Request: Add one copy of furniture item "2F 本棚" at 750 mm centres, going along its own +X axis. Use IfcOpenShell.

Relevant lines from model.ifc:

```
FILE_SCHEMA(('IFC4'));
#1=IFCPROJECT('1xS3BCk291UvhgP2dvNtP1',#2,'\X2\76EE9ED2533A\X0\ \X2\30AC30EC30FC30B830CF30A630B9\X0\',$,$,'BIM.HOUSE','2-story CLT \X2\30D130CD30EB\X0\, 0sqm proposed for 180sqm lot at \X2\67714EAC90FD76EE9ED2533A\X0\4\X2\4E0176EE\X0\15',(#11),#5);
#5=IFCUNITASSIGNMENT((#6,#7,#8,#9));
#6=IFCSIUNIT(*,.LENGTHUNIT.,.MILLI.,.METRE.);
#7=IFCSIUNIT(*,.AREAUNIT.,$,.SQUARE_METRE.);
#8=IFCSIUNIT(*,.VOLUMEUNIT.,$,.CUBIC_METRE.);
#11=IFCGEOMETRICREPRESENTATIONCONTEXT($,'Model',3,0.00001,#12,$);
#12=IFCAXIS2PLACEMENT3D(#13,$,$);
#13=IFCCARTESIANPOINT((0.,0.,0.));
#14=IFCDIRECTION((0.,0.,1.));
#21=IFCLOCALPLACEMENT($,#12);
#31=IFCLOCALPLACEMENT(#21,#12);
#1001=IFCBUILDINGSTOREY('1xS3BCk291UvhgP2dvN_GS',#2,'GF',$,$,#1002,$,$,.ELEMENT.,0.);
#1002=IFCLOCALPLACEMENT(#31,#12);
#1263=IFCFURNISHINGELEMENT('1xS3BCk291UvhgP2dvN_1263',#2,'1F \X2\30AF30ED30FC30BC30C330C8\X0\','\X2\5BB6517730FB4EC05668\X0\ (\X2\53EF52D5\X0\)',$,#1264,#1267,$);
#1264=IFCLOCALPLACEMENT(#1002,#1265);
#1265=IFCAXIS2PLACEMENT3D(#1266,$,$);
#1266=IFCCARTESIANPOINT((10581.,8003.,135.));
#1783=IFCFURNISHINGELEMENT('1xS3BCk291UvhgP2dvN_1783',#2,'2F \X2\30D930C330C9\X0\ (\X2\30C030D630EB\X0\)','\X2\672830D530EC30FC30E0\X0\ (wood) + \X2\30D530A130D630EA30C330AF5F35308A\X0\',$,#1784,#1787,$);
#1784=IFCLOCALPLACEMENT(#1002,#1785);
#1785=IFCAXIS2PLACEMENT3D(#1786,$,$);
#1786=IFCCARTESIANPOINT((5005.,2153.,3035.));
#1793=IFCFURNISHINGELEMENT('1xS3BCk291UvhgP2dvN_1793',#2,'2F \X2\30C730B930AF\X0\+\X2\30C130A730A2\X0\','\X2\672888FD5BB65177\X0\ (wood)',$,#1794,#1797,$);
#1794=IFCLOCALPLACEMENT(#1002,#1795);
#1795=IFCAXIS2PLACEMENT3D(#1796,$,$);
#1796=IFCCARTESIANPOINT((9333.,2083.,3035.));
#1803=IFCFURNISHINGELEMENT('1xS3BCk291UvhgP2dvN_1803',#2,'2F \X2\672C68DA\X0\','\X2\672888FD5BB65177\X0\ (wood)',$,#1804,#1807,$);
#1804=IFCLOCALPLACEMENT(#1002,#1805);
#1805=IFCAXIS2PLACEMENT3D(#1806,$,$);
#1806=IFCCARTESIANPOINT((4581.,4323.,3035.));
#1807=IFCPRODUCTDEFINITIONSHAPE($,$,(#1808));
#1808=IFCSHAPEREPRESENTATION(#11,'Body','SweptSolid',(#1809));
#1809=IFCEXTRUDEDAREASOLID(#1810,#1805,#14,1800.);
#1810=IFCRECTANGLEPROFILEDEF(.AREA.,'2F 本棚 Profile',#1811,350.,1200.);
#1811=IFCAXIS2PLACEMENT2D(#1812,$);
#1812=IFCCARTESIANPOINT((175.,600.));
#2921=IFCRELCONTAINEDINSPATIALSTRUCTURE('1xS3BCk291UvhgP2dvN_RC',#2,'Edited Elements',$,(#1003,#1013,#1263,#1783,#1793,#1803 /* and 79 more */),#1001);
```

```python
import ifcopenshell
import ifcopenshell.api.geometry
import ifcopenshell.api.root
import ifcopenshell.util.element
import ifcopenshell.util.placement

model = ifcopenshell.open("model.ifc")


def reuse_history(source, copy):
    """copy_class also copies each property set's owner history, people and application; keep the originals."""
    for rel in copy.IsDefinedBy:
        if rel.is_a("IfcRelDefinesByProperties") and (history := rel.RelatingPropertyDefinition.OwnerHistory):
            rel.RelatingPropertyDefinition.OwnerHistory = source.OwnerHistory
            ifcopenshell.util.element.remove_deep2(model, history)


source = model.by_id(1803)
base = ifcopenshell.util.placement.get_local_placement(source.ObjectPlacement)
step = base[:3, 0] * 750.0

for i in range(1, 2):
    copy = ifcopenshell.api.root.copy_class(model, product=source)
    copy.Representation = ifcopenshell.util.element.copy_deep(
        model, source.Representation, exclude=["IfcGeometricRepresentationContext", "IfcRepresentationMap"]
    )
    reuse_history(source, copy)
    matrix = base.copy()
    matrix[:3, 3] += i * step
    print("added at", matrix[:3, 3].round(3) + 0.0)
    ifcopenshell.api.geometry.edit_object_placement(model, product=copy, matrix=matrix, is_si=False)

model.write("model_v2.ifc")
```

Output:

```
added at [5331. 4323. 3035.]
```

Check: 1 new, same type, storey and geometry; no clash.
